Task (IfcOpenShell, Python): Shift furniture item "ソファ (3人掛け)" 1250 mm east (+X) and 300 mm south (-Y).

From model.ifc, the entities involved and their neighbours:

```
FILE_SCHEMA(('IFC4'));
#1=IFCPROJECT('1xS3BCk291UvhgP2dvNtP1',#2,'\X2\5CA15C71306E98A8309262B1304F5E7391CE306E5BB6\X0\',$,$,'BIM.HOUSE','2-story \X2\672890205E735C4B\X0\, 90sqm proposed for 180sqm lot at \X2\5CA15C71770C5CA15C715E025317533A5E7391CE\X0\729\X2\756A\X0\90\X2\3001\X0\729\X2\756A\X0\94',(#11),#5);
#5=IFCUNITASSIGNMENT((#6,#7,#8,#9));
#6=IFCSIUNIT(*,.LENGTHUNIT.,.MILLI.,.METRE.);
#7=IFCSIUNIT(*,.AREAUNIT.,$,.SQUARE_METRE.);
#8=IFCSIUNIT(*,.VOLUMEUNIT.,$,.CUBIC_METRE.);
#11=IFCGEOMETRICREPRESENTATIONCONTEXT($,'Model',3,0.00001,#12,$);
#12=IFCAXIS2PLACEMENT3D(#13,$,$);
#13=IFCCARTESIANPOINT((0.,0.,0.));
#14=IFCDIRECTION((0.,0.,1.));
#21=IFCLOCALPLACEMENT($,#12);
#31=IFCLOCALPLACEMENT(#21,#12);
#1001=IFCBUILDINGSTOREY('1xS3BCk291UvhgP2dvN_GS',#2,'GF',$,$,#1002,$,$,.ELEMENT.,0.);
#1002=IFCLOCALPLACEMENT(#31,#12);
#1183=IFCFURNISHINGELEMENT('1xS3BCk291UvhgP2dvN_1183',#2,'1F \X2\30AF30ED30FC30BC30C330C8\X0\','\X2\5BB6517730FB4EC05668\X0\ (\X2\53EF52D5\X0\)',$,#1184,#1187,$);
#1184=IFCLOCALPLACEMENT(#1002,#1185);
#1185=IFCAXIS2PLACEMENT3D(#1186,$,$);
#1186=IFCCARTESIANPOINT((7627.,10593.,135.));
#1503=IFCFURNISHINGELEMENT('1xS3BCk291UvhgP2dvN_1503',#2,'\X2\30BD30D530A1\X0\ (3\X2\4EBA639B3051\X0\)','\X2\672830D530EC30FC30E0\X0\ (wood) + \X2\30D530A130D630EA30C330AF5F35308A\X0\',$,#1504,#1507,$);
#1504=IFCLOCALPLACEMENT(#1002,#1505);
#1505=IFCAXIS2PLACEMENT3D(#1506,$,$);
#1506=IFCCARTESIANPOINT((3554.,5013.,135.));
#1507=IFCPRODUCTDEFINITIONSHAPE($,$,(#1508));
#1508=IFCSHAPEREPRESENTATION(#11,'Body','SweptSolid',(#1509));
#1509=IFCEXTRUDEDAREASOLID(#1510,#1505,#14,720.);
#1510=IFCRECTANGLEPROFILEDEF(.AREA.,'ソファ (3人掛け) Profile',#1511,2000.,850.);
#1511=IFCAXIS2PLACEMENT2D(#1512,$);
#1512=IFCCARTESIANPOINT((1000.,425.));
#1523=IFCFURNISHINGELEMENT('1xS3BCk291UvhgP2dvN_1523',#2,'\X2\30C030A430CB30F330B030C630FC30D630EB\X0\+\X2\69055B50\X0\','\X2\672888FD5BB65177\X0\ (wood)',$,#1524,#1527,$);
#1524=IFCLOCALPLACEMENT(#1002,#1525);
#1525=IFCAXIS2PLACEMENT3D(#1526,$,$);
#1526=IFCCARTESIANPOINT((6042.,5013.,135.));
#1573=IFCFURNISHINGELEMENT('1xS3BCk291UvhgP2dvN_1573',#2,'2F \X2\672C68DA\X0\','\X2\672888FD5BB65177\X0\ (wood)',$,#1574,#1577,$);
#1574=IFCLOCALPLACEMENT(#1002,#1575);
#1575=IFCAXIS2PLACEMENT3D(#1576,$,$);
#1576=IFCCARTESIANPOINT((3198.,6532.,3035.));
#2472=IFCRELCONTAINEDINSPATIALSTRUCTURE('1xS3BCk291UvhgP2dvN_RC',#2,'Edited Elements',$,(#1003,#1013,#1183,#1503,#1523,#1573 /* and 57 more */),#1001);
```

```python
import ifcopenshell
import ifcopenshell.api.geometry
import ifcopenshell.util.placement
import ifcopenshell.util.unit

model = ifcopenshell.open("model.ifc")
unit_scale = ifcopenshell.util.unit.calculate_unit_scale(model)

item = model.by_guid("1xS3BCk291UvhgP2dvN_1503")
matrix = ifcopenshell.util.placement.get_local_placement(item.ObjectPlacement)
matrix[0, 3] += 1.25 / unit_scale
matrix[1, 3] -= 0.3 / unit_scale
ifcopenshell.api.geometry.edit_object_placement(model, product=item, matrix=matrix, is_si=False)

print(ifcopenshell.util.placement.get_local_placement(item.ObjectPlacement).round(3) + 0.0)

model.write("model_v2.ifc")
```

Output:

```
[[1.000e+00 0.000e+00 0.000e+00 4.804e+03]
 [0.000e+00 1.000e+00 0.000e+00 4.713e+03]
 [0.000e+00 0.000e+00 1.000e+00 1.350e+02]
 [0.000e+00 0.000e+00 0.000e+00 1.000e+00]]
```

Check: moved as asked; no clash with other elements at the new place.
